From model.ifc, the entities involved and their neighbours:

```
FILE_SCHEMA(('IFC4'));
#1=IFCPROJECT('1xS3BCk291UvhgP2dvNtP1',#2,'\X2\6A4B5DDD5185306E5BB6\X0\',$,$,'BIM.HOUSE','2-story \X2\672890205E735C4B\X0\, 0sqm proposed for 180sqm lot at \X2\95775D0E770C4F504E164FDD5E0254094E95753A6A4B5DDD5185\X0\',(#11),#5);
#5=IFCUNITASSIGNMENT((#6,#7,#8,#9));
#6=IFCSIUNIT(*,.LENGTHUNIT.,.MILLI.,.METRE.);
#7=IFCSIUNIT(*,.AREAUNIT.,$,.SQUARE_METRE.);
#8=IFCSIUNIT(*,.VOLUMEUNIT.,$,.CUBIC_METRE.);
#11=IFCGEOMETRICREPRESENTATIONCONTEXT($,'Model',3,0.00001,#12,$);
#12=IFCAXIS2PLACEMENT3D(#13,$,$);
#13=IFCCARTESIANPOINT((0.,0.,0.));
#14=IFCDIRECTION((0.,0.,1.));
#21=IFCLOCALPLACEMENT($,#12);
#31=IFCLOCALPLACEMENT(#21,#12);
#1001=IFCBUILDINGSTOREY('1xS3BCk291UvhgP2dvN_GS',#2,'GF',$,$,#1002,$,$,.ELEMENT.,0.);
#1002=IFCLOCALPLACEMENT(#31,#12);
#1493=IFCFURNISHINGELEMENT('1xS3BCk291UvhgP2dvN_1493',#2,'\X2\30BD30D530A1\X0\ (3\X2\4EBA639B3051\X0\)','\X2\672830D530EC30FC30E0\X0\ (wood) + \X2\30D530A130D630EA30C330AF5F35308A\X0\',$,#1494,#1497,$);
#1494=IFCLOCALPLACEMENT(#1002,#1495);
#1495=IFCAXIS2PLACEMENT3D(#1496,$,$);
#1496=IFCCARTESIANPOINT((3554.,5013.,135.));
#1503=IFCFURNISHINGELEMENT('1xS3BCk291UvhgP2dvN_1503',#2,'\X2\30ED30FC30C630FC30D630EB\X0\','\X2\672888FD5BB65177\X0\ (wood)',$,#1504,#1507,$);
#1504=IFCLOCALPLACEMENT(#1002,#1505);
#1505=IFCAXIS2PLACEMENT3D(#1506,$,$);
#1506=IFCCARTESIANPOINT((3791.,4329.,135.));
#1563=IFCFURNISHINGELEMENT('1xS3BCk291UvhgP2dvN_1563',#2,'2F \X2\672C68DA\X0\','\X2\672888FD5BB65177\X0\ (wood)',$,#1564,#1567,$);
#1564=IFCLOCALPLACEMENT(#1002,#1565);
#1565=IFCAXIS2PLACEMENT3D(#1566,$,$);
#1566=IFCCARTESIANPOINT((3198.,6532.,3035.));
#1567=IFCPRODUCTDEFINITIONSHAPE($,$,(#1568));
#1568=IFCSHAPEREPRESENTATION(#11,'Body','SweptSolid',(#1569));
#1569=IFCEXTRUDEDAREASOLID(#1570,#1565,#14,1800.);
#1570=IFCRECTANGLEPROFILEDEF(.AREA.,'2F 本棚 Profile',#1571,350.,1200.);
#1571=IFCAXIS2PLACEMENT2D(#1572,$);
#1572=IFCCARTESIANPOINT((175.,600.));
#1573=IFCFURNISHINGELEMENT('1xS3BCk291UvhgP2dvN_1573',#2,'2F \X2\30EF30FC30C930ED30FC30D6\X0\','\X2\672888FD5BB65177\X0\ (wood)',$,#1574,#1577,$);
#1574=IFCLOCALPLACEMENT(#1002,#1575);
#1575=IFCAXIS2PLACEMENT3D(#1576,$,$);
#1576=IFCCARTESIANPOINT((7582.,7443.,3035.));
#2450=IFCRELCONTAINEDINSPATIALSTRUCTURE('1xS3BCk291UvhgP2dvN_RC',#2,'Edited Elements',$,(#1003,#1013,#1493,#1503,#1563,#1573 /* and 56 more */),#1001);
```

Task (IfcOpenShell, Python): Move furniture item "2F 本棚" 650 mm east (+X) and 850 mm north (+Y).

```python
import ifcopenshell
import ifcopenshell.api.geometry
import ifcopenshell.util.placement

model = ifcopenshell.open("model.ifc")

item = model.by_guid("1xS3BCk291UvhgP2dvN_1563")
matrix = ifcopenshell.util.placement.get_local_placement(item.ObjectPlacement)
matrix[0, 3] += 650.0
matrix[1, 3] += 850.0
ifcopenshell.api.geometry.edit_object_placement(model, product=item, matrix=matrix, is_si=False)

print(ifcopenshell.util.placement.get_local_placement(item.ObjectPlacement).round(3) + 0.0)

model.write("model_rev.ifc")
```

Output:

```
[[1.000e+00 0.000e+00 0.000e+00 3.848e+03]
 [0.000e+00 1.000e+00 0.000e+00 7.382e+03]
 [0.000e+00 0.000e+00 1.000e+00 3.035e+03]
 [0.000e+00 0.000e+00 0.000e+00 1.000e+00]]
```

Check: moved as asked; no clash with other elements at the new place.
